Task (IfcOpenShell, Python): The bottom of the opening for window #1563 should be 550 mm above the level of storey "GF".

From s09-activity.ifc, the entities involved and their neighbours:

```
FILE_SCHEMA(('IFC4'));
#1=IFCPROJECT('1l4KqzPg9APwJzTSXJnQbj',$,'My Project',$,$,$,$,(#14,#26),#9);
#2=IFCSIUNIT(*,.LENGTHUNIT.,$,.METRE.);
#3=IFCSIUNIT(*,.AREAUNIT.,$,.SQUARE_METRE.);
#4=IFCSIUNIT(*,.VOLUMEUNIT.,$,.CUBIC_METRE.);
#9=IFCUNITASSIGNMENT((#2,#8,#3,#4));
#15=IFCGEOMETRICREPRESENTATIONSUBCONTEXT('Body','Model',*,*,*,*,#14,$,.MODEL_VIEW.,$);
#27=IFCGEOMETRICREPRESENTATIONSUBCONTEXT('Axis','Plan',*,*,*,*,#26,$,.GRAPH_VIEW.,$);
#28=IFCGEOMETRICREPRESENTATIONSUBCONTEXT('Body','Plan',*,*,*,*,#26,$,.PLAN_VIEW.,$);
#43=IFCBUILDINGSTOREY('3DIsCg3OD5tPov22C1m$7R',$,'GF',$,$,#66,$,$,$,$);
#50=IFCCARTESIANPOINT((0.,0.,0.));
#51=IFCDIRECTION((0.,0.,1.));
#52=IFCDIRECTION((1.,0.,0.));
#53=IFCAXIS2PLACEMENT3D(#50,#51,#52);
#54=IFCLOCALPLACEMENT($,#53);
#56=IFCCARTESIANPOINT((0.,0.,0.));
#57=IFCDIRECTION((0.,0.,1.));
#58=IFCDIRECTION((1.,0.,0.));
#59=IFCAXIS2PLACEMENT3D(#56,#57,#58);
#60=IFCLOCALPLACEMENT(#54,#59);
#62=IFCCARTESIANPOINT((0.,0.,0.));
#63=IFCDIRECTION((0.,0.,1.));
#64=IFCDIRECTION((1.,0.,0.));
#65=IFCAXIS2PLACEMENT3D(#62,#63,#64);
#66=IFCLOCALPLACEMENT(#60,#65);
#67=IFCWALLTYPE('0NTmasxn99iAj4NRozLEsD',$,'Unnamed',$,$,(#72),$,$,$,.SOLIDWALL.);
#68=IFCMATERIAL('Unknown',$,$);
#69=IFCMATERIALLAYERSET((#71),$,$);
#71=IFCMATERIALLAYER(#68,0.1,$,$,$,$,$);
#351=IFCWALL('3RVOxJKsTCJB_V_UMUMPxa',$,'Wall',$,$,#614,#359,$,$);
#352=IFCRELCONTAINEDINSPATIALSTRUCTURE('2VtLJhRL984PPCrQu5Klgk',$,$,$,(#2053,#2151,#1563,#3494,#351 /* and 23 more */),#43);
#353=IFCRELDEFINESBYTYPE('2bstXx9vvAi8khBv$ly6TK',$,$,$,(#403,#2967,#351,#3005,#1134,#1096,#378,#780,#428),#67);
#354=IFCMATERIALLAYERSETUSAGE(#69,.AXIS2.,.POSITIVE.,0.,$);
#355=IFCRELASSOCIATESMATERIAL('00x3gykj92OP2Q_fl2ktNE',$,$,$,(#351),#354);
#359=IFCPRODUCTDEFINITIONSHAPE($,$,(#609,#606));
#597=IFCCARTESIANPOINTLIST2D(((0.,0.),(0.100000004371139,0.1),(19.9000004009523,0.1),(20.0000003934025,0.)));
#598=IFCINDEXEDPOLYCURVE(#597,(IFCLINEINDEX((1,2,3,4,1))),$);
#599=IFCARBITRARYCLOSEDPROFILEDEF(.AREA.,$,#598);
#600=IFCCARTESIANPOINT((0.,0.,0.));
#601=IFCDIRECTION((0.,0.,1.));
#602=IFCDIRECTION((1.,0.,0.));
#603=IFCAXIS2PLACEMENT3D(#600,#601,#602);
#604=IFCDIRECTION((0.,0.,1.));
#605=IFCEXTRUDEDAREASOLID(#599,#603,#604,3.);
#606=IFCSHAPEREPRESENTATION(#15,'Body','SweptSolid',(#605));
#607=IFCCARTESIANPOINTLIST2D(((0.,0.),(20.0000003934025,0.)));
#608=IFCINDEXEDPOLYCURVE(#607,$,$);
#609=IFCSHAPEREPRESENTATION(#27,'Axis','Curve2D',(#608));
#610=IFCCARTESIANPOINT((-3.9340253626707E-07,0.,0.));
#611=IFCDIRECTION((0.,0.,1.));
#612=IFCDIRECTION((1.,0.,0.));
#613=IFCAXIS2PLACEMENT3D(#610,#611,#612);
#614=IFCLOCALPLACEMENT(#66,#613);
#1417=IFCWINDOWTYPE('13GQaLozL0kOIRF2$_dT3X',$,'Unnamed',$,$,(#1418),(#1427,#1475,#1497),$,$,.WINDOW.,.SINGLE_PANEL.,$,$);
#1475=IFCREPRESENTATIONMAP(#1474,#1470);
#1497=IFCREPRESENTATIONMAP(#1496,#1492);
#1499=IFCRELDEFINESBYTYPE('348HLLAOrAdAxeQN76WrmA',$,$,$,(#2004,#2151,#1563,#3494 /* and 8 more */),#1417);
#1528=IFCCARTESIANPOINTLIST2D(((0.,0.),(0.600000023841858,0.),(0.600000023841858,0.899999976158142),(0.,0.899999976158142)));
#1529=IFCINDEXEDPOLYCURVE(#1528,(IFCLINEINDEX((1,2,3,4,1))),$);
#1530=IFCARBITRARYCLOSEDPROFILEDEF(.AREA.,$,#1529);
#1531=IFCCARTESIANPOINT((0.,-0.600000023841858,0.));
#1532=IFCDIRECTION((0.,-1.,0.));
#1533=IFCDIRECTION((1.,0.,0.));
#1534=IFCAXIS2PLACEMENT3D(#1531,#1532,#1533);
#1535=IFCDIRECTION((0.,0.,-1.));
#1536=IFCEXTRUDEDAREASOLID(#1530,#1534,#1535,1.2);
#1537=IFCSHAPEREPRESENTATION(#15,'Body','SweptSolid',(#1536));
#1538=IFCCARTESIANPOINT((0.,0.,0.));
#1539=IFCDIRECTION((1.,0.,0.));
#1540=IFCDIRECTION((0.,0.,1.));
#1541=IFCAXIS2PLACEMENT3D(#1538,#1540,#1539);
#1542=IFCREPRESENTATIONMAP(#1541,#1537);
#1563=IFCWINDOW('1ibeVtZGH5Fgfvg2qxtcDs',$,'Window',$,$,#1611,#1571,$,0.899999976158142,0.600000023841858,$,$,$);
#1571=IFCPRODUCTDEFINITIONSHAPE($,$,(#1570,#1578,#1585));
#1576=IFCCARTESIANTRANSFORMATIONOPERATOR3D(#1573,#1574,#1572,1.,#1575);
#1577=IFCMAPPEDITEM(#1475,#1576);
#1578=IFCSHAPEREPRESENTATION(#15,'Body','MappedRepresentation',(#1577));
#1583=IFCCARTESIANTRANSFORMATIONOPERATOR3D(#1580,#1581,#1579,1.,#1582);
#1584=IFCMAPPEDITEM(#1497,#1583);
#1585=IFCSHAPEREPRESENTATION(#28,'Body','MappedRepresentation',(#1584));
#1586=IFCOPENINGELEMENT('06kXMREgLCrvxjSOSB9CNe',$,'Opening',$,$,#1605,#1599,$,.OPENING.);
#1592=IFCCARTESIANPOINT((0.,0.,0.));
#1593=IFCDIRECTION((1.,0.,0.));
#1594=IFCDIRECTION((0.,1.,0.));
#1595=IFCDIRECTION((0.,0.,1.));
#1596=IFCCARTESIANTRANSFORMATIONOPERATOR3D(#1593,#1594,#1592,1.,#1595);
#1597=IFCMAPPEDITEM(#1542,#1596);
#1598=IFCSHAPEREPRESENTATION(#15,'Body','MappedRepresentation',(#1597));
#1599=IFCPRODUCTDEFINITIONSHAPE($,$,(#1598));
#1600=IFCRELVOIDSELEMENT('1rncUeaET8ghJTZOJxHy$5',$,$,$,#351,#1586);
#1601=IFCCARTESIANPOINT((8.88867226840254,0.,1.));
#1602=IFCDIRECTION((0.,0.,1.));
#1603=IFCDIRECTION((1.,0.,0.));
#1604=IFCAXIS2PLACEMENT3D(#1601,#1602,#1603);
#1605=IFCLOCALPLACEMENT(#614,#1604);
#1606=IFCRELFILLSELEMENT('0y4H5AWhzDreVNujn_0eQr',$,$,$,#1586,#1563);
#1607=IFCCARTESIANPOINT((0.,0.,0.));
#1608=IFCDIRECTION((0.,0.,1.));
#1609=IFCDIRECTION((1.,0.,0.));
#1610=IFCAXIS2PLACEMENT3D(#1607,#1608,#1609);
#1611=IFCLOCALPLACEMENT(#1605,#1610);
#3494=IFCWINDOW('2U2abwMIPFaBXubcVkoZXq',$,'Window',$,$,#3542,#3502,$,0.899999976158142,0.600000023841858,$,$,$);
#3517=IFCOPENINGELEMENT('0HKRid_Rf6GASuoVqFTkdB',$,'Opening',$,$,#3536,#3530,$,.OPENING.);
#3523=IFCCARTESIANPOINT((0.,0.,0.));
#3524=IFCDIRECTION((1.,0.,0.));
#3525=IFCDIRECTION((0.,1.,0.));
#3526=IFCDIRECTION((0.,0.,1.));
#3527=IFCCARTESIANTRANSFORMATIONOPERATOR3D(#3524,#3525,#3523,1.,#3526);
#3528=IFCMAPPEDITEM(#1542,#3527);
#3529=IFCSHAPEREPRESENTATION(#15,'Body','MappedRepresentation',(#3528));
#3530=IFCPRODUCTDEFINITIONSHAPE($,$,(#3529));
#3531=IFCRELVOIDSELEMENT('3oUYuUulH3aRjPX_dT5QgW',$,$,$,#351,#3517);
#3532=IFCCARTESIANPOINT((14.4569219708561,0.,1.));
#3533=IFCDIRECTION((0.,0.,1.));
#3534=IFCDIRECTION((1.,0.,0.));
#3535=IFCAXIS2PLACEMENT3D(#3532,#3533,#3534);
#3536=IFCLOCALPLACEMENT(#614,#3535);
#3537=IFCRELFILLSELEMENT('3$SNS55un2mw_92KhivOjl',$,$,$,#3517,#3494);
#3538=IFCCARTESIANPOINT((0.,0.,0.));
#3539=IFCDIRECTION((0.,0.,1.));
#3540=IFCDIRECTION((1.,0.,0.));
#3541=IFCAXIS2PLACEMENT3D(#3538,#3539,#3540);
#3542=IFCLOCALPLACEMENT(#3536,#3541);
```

```python
import numpy as np
import ifcopenshell
import ifcopenshell.api.geometry
import ifcopenshell.geom
import ifcopenshell.util.element
import ifcopenshell.util.placement
import ifcopenshell.util.shape
import ifcopenshell.util.unit

model = ifcopenshell.open("s09-activity.ifc")
unit_scale = ifcopenshell.util.unit.calculate_unit_scale(model)

window = model.by_guid("1ibeVtZGH5Fgfvg2qxtcDs")
opening = window.FillsVoids[0].RelatingOpeningElement
storey = ifcopenshell.util.element.get_container(window, ifc_class="IfcBuildingStorey")
level = ifcopenshell.util.placement.get_local_placement(storey.ObjectPlacement)[2, 3]

# The opening's origin need not be at the sill, so measure its lowest point.
shape = ifcopenshell.geom.create_shape(ifcopenshell.geom.settings(), opening)
bottom = ifcopenshell.util.shape.get_shape_bottom_elevation(shape, shape.geometry) / unit_scale
dz = level + 0.55 - bottom

shift = np.array([0.0, 0.0, dz])
# The window is placed relative to its opening, so it follows when the opening moves.
matrix = ifcopenshell.util.placement.get_local_placement(opening.ObjectPlacement)
matrix[:3, 3] += shift
ifcopenshell.api.geometry.edit_object_placement(
    model, product=opening, matrix=matrix, is_si=False, should_transform_children=True
)

print(f"moved by {dz * unit_scale:+.3f} m")

model.write("s09-activity_v2.ifc")
```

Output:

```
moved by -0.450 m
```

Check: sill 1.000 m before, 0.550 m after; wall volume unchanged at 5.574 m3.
